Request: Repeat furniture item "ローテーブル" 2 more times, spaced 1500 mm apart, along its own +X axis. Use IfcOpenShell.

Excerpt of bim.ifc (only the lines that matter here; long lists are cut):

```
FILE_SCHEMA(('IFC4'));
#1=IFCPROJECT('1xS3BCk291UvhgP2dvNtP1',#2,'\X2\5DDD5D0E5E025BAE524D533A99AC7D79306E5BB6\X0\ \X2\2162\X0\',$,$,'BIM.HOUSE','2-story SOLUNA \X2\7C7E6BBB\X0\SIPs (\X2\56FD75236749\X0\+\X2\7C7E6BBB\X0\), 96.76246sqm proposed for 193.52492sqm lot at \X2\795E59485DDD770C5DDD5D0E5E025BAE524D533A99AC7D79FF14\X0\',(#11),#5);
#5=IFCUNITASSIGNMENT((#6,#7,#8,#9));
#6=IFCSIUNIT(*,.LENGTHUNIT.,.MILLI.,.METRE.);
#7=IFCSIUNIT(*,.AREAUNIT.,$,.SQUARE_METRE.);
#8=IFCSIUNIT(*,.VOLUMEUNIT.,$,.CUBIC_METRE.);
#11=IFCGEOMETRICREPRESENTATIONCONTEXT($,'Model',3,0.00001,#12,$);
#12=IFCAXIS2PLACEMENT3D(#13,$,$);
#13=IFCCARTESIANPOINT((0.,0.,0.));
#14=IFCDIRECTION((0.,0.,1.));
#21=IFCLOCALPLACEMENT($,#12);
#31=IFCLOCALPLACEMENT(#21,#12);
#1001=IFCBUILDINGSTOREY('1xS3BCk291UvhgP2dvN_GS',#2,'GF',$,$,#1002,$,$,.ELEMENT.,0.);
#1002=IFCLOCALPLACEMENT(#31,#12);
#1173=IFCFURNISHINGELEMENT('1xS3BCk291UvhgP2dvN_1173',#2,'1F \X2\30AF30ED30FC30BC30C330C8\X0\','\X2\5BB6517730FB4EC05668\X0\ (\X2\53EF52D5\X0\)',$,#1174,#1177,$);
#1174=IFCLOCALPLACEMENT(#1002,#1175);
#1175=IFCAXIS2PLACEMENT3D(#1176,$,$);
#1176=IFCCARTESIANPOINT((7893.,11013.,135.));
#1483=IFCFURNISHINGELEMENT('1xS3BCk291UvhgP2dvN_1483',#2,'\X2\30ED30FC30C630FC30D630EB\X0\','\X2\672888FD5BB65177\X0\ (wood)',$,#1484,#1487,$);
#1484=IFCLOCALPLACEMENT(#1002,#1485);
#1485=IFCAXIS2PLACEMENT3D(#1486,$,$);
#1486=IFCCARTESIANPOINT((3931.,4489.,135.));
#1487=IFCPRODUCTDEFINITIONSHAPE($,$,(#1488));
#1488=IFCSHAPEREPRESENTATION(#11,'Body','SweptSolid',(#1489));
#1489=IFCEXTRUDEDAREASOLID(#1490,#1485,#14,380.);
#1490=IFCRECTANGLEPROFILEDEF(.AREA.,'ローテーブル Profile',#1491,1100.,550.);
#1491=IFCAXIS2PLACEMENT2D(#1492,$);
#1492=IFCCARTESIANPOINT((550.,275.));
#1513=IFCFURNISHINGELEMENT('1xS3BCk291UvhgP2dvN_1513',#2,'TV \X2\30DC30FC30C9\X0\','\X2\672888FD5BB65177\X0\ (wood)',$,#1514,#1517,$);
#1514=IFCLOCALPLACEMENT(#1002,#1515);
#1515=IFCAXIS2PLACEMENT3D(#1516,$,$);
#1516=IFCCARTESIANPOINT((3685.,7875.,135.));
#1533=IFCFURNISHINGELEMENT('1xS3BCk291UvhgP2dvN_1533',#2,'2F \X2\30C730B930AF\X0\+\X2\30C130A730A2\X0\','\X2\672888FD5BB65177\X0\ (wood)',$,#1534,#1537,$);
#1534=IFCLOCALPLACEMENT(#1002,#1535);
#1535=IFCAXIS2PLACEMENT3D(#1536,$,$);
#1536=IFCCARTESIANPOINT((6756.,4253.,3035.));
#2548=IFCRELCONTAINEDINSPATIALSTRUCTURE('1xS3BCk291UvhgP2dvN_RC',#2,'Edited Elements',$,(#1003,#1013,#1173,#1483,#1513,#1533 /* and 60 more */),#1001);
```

```python
import ifcopenshell
import ifcopenshell.api.geometry
import ifcopenshell.api.root
import ifcopenshell.util.element
import ifcopenshell.util.placement
import ifcopenshell.util.unit

model = ifcopenshell.open("bim.ifc")
unit_scale = ifcopenshell.util.unit.calculate_unit_scale(model)


def reuse_history(source, copy):
    """copy_class also copies each property set's owner history, people and application; keep the originals."""
    for rel in copy.IsDefinedBy:
        if rel.is_a("IfcRelDefinesByProperties") and (history := rel.RelatingPropertyDefinition.OwnerHistory):
            rel.RelatingPropertyDefinition.OwnerHistory = source.OwnerHistory
            ifcopenshell.util.element.remove_deep2(model, history)


source = model.by_id(1483)
base = ifcopenshell.util.placement.get_local_placement(source.ObjectPlacement)
step = base[:3, 0] * 1.5 / unit_scale

for i in range(1, 3):
    copy = ifcopenshell.api.root.copy_class(model, product=source)
    copy.Representation = ifcopenshell.util.element.copy_deep(
        model, source.Representation, exclude=["IfcGeometricRepresentationContext", "IfcRepresentationMap"]
    )
    reuse_history(source, copy)
    matrix = base.copy()
    matrix[:3, 3] += i * step
    print("added at", matrix[:3, 3].round(3) + 0.0)
    ifcopenshell.api.geometry.edit_object_placement(model, product=copy, matrix=matrix, is_si=False)

model.write("bim-out.ifc")
```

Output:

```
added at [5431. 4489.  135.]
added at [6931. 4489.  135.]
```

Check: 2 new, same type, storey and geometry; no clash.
